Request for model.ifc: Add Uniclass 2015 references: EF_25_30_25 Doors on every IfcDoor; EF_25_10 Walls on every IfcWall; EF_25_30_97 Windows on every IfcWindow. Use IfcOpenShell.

First a look at what the model holds.

```python
import ifcopenshell

model = ifcopenshell.open("model.ifc")
print(model.schema)
print("classifications:", [c.Name for c in model.by_type("IfcClassification")])
for ifc_class in ("IfcDoor", "IfcRoof", "IfcStair", "IfcWall", "IfcWindow"):
    print(ifc_class, len(model.by_type(ifc_class)))
```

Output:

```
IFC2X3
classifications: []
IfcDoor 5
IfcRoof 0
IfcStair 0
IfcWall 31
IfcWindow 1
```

```python
import ifcopenshell
import ifcopenshell.api.classification

model = ifcopenshell.open("model.ifc")

# IFC2X3 requires Source and Edition and has no link from the project to the system.
system = model.create_entity("IfcClassification", Source="NBS", Edition="2015", Name="Uniclass 2015")

codes = {
    "IfcDoor": ("EF_25_30_25", "Doors"),
    "IfcWall": ("EF_25_10", "Walls"),
    "IfcWindow": ("EF_25_30_97", "Windows"),
}
for ifc_class, (code, name) in codes.items():
    products = model.by_type(ifc_class)
    ifcopenshell.api.classification.add_reference(
        model, products=products, classification=system, identification=code, name=name
    )
    print(code, len(products))

model.write("model_edited.ifc")
```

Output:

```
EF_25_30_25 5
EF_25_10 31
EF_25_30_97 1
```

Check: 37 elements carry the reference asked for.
